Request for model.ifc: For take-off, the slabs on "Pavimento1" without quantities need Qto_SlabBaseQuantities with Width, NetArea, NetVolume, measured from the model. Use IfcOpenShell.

First a look at what the model holds.

```python
import ifcopenshell
import ifcopenshell.util.element
import ifcopenshell.util.unit

model = ifcopenshell.open("model.ifc")
print(model.schema)
for unit_type in ("LENGTHUNIT", "AREAUNIT", "VOLUMEUNIT"):
    print(unit_type, ifcopenshell.util.unit.calculate_unit_scale(model, unit_type))
storey = next(s for s in model.by_type("IfcBuildingStorey") if s.Name == "Pavimento1")
slabs = [e for e in ifcopenshell.util.element.get_decomposition(storey) if e.is_a("IfcSlab")]
for e in sorted(slabs, key=lambda e: e.id()):
    print(e.id(), e.is_a(), e.Name, list(ifcopenshell.util.element.get_psets(e, qtos_only=True)), sep=" | ")
```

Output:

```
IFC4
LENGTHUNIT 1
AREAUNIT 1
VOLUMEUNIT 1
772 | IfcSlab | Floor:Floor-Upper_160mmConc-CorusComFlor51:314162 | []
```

```python
import ifcopenshell
import ifcopenshell.api.pset
import ifcopenshell.geom
import ifcopenshell.util.element
import ifcopenshell.util.shape
import ifcopenshell.util.unit

model = ifcopenshell.open("model.ifc")
unit_scale = ifcopenshell.util.unit.calculate_unit_scale(model)
area_scale = ifcopenshell.util.unit.calculate_unit_scale(model, "AREAUNIT")
volume_scale = ifcopenshell.util.unit.calculate_unit_scale(model, "VOLUMEUNIT")
settings = ifcopenshell.geom.settings()

storey = next(s for s in model.by_type("IfcBuildingStorey") if s.Name == "Pavimento1")
slabs = [e for e in ifcopenshell.util.element.get_decomposition(storey) if e.is_a("IfcSlab")]

for e in sorted(slabs, key=lambda e: e.id()):
    if ifcopenshell.util.element.get_psets(e, qtos_only=True, should_inherit=False):
        continue
    # Geometry comes back in metres, in the element's own axes.
    shape = ifcopenshell.geom.create_shape(settings, e)
    values = {
        "Width": ifcopenshell.util.shape.get_z(shape.geometry) / unit_scale,
        "NetArea": ifcopenshell.util.shape.get_footprint_area(shape.geometry) / area_scale,
        "NetVolume": ifcopenshell.util.shape.get_volume(shape.geometry) / volume_scale,
    }
    qto = ifcopenshell.api.pset.add_qto(model, product=e, name="Qto_SlabBaseQuantities")
    ifcopenshell.api.pset.edit_qto(model, qto=qto, properties=values)
    print(e.id(), {k: round(v, 3) for k, v in values.items()})

model.write("model_v2.ifc")
```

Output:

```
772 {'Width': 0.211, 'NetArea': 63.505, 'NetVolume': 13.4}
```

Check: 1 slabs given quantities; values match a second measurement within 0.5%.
